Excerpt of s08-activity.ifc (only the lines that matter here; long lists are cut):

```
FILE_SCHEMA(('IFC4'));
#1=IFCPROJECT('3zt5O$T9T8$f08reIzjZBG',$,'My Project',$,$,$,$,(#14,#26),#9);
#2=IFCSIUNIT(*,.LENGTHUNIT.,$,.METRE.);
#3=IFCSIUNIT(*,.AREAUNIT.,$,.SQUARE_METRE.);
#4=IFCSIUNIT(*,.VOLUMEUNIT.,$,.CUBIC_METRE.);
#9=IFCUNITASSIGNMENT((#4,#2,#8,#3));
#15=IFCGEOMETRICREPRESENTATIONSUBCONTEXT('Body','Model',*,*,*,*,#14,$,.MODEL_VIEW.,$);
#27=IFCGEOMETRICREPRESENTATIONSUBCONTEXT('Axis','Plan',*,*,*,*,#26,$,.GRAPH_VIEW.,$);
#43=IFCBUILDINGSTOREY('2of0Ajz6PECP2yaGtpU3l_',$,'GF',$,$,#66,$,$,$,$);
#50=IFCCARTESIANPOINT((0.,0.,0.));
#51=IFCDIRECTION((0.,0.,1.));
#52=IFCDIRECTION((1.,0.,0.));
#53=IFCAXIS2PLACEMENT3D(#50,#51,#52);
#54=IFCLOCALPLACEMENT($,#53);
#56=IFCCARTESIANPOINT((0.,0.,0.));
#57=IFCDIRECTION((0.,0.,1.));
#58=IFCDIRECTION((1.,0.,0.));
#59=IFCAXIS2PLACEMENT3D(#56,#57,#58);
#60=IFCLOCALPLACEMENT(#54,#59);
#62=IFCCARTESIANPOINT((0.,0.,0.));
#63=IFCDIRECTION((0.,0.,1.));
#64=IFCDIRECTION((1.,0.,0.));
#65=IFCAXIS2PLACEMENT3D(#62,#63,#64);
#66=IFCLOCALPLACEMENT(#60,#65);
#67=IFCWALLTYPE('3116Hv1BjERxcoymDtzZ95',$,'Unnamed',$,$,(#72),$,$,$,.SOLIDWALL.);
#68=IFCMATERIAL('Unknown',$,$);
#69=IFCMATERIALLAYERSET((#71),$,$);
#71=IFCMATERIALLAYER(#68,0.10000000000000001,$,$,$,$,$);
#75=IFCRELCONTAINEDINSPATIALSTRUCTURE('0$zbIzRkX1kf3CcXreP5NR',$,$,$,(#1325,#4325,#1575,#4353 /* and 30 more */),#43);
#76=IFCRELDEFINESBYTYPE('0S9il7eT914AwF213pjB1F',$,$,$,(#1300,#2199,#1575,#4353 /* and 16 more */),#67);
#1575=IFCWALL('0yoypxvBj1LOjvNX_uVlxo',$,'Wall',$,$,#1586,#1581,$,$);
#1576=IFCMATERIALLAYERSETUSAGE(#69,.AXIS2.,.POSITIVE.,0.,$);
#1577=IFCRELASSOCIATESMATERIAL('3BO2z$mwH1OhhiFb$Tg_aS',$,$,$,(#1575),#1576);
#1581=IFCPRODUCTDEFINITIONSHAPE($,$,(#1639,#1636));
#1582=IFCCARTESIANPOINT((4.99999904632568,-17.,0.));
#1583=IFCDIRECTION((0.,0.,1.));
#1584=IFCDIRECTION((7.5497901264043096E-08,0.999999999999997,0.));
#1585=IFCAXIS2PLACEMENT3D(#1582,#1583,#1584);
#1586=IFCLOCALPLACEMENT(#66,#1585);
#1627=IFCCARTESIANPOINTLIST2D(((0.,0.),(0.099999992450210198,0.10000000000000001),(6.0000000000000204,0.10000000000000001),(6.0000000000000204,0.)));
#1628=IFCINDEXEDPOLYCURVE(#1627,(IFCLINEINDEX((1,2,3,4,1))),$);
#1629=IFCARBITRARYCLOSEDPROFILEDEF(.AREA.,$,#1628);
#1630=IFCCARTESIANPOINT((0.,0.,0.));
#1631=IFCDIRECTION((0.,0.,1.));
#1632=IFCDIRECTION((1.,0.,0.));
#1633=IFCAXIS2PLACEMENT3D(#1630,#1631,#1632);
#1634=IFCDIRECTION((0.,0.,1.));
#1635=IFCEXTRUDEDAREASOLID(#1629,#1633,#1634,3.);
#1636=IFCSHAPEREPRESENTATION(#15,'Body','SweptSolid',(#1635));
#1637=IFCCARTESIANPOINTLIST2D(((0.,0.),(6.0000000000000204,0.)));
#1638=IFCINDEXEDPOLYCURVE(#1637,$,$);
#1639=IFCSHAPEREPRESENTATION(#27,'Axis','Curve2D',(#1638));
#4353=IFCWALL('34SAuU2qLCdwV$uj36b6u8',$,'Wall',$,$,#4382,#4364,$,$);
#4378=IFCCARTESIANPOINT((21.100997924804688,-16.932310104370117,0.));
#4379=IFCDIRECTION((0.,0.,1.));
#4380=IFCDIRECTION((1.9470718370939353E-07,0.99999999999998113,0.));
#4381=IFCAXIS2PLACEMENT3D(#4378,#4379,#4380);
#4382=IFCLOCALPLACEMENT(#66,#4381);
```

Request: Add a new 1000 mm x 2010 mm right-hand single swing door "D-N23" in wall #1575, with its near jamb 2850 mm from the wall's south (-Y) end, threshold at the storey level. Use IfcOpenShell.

```python
import numpy as np
import ifcopenshell
import ifcopenshell.api.feature
import ifcopenshell.api.geometry
import ifcopenshell.api.root
import ifcopenshell.api.spatial
import ifcopenshell.geom
import ifcopenshell.util.element
import ifcopenshell.util.placement
import ifcopenshell.util.representation
import ifcopenshell.util.shape
import ifcopenshell.util.unit

model = ifcopenshell.open("s08-activity.ifc")
unit_scale = ifcopenshell.util.unit.calculate_unit_scale(model)
settings = ifcopenshell.geom.settings()


def volume(element):
    """Net volume in cubic metres, openings subtracted."""
    shape = ifcopenshell.geom.create_shape(settings, element)
    return ifcopenshell.util.shape.get_volume(shape.geometry)


wall = model.by_id(1575)
storey = ifcopenshell.util.element.get_container(wall, ifc_class="IfcBuildingStorey")
context = ifcopenshell.util.representation.get_context(model, "Model", "Body", "MODEL_VIEW")
before = volume(wall)

width, height, from_end, sill = 1, 2.01, 2.85, 0.0  # metres

# The wall runs along its own X axis, and the end named is its -X end.
wall_shape = ifcopenshell.geom.create_shape(settings, wall)
x, y, z = ifcopenshell.util.shape.get_vertices(wall_shape.geometry).T
start = x.min() + from_end
face, thickness = float(y.min()), float(y.max() - y.min())
wall_matrix = ifcopenshell.util.placement.get_local_placement(wall.ObjectPlacement)
level = ifcopenshell.util.placement.get_local_placement(storey.ObjectPlacement)[2, 3]


def in_wall(x, y):
    """Placement at x, y metres in the wall's axes, at sill height."""
    matrix = wall_matrix.copy()
    matrix[:, 3] = wall_matrix @ np.array([x / unit_scale, y / unit_scale, 0.0, 1.0])
    matrix[2, 3] = level + sill / unit_scale
    return matrix


# Opening: a box that overshoots both wall faces by 50 mm.
opening = ifcopenshell.api.root.create_entity(model, ifc_class="IfcOpeningElement", predefined_type="OPENING")
box = ifcopenshell.api.geometry.add_wall_representation(
    model, context=context, length=width, height=height, thickness=thickness + 0.1
)
ifcopenshell.api.geometry.assign_representation(model, product=opening, representation=box)
ifcopenshell.api.geometry.edit_object_placement(model, product=opening, matrix=in_wall(start, face - 0.05), is_si=False)
ifcopenshell.api.feature.add_feature(model, feature=opening, element=wall)

door = ifcopenshell.api.root.create_entity(model, ifc_class="IfcDoor", name="D-N23", predefined_type="DOOR")
door.OverallWidth, door.OverallHeight = width / unit_scale, height / unit_scale
door.OperationType = "SINGLE_SWING_RIGHT"
body = ifcopenshell.api.geometry.add_door_representation(
    model,
    context=context,
    overall_width=door.OverallWidth,
    overall_height=door.OverallHeight,
    operation_type="SINGLE_SWING_RIGHT",
    lining_properties={"LiningDepth": thickness / unit_scale, "ThresholdDepth": thickness / unit_scale},
)
ifcopenshell.api.geometry.assign_representation(model, product=door, representation=body)
ifcopenshell.api.spatial.assign_container(model, products=[door], relating_structure=storey)
ifcopenshell.api.feature.add_filling(model, opening=opening, element=door)

# The lining spans the wall, so the door starts at the wall face.
ifcopenshell.api.geometry.edit_object_placement(model, product=door, matrix=in_wall(start, face), is_si=False)

after = volume(wall)

print(f"wall volume {before:.3f} -> {after:.3f} m3")

model.write("s08-activity_v2.ifc")
```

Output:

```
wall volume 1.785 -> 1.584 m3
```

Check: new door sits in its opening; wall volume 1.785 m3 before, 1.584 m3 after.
